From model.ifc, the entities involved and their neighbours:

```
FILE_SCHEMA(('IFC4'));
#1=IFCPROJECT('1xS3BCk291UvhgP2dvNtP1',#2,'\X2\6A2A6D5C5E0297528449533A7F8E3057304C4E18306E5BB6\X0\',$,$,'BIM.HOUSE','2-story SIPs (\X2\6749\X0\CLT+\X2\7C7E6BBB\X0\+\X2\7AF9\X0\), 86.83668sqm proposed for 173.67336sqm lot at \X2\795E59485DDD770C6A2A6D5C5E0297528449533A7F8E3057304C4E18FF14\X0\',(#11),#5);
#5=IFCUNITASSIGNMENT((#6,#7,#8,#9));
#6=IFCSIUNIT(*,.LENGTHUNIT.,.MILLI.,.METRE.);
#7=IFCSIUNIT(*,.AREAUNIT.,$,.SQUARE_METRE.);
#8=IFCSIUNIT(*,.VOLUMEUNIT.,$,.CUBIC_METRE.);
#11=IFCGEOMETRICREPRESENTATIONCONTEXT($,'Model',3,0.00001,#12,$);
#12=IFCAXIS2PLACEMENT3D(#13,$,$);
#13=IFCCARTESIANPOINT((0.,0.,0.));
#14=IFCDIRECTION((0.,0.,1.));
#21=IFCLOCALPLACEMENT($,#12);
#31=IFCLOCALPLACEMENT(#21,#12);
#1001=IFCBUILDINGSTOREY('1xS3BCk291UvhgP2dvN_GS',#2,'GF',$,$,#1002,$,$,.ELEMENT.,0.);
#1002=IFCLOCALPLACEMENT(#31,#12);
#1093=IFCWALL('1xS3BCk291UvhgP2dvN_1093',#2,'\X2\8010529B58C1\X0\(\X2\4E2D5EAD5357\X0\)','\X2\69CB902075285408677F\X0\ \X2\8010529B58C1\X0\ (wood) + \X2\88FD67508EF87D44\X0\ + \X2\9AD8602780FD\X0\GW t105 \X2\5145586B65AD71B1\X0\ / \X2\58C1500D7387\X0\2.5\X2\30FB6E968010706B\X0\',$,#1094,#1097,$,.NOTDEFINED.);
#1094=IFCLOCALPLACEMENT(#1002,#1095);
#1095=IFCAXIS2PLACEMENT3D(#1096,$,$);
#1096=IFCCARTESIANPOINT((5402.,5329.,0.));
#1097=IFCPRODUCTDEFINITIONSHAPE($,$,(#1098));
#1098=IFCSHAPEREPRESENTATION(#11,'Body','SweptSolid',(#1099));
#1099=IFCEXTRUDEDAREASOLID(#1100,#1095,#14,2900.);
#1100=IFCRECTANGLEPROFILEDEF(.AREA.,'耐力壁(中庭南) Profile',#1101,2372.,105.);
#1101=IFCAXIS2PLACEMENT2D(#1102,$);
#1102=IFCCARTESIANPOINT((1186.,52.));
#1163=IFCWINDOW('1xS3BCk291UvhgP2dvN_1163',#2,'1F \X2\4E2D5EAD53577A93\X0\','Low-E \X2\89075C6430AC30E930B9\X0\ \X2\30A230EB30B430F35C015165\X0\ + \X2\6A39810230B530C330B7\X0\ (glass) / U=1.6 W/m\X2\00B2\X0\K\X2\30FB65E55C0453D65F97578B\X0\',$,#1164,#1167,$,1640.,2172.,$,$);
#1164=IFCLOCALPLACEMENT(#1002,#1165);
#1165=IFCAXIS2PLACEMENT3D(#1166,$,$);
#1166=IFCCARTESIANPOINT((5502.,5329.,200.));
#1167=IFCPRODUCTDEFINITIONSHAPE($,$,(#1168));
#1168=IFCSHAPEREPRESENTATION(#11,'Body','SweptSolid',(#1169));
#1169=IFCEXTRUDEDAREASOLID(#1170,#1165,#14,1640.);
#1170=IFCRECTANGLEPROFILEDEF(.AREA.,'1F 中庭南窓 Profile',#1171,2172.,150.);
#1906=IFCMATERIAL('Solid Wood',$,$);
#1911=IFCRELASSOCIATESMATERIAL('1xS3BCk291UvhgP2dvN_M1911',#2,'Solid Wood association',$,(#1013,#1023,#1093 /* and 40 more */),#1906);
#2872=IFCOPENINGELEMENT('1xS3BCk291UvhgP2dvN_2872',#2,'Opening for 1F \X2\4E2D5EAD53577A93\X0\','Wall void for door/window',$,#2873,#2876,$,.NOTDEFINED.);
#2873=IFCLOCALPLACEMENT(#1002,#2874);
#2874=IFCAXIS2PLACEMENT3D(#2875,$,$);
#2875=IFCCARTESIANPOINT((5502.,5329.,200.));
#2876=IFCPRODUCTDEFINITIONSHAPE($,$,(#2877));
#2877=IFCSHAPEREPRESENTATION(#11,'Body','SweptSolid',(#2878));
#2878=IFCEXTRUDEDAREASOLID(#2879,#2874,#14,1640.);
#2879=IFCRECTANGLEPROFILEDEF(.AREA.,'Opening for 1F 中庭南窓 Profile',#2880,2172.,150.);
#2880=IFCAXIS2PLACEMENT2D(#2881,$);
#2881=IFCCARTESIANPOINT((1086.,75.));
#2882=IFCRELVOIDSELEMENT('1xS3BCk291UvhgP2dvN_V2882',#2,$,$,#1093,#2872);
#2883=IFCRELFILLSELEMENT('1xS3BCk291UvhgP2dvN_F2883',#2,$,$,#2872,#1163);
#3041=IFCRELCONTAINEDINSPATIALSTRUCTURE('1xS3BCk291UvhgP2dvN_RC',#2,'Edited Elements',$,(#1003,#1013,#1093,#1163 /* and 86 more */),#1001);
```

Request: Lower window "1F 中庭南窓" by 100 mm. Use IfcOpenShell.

```python
import numpy as np
import ifcopenshell
import ifcopenshell.api.geometry
import ifcopenshell.util.placement
import ifcopenshell.util.unit

model = ifcopenshell.open("model.ifc")
unit_scale = ifcopenshell.util.unit.calculate_unit_scale(model)

window = model.by_guid("1xS3BCk291UvhgP2dvN_1163")
opening = window.FillsVoids[0].RelatingOpeningElement
dz = -0.1 / unit_scale

shift = np.array([0.0, 0.0, dz])
# The window is not placed relative to its opening, so move both.
for product in (opening, window):
    matrix = ifcopenshell.util.placement.get_local_placement(product.ObjectPlacement)
    matrix[:3, 3] += shift
    ifcopenshell.api.geometry.edit_object_placement(model, product=product, matrix=matrix, is_si=False)

print(f"moved by {dz * unit_scale:+.3f} m")

model.write("model_rev.ifc")
```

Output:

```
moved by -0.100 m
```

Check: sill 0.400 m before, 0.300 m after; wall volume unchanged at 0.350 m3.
